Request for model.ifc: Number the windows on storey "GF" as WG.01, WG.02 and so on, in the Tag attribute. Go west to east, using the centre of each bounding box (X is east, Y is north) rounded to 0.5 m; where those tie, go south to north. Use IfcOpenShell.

First a look at what the model holds.

```python
import ifcopenshell
import ifcopenshell.util.element
import ifcopenshell.util.placement

model = ifcopenshell.open("model.ifc")
print(model.schema)
storey = next(s for s in model.by_type("IfcBuildingStorey") if s.Name == "GF")
windows = [e for e in ifcopenshell.util.element.get_decomposition(storey) if e.is_a("IfcWindow")]
for e in sorted(windows, key=lambda e: e.id()):
    origin = ifcopenshell.util.placement.get_local_placement(e.ObjectPlacement)[:3, 3]
    print(e.id(), e.Tag, e.Name, origin.round(2) + 0.0, sep=" | ")
```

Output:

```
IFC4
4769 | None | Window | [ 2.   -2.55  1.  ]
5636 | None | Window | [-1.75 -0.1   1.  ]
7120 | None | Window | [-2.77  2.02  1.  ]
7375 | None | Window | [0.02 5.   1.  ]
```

```python
import ifcopenshell
import ifcopenshell.geom
import ifcopenshell.util.element
import ifcopenshell.util.shape

model = ifcopenshell.open("model.ifc")
settings = ifcopenshell.geom.settings()
settings.set("use-world-coords", True)


def centre(element):
    shape = ifcopenshell.geom.create_shape(settings, element)
    return ifcopenshell.util.shape.get_bbox_centroid(shape.geometry)


storey = next(s for s in model.by_type("IfcBuildingStorey") if s.Name == "GF")
windows = [e for e in ifcopenshell.util.element.get_decomposition(storey) if e.is_a("IfcWindow")]

# Insertion points can sit at a corner or the storey origin, so sort by the geometry (in metres).
centres = {e: centre(e) for e in windows}
windows.sort(key=lambda e: (round(centres[e][0] / 0.5), centres[e][1]))

for i, e in enumerate(windows, start=1):
    number = f"WG.{i:02d}"
    e.Tag = number
    print(e.id(), number)

model.write("model_updated.ifc")
```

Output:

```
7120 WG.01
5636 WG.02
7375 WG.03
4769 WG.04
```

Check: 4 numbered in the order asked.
